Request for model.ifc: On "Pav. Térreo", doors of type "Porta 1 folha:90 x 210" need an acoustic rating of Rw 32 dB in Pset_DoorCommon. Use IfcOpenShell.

First a look at what the model holds.

```python
import ifcopenshell
import ifcopenshell.util.element

model = ifcopenshell.open("model.ifc")
print(model.schema)
storey = next(s for s in model.by_type("IfcBuildingStorey") if s.Name == "Pav. Térreo")
doors = [e for e in ifcopenshell.util.element.get_decomposition(storey) if e.is_a("IfcDoor")]
seen = {}
for e in doors:
    element_type = ifcopenshell.util.element.get_type(e)
    key = (element_type.Name if element_type != e and element_type else None, ifcopenshell.util.element.get_pset(e, "Pset_DoorCommon", "AcousticRating"))
    seen[key] = seen.get(key, 0) + 1
for (name, value), count in sorted(seen.items(), key=str):
    print(count, "x", name, "|", value)
```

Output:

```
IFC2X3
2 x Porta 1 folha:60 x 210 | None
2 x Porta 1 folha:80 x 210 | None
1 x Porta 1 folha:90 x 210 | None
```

```python
import ifcopenshell
import ifcopenshell.api.pset
import ifcopenshell.util.element

model = ifcopenshell.open("model.ifc")

storey = next(s for s in model.by_type("IfcBuildingStorey") if s.Name == "Pav. Térreo")
doors = [e for e in ifcopenshell.util.element.get_decomposition(storey) if e.is_a("IfcDoor")]

count = 0
for e in doors:
    element_type = ifcopenshell.util.element.get_type(e)
    if element_type in (None, e) or element_type.Name != "Porta 1 folha:90 x 210":
        continue
    # add_pset returns the element's existing set when there is one.
    pset = ifcopenshell.api.pset.add_pset(model, product=e, name="Pset_DoorCommon")
    ifcopenshell.api.pset.edit_pset(model, pset=pset, properties={"AcousticRating": "Rw 32 dB"})
    count += 1

print(count, "doors updated")

model.write("model_v2.ifc")
```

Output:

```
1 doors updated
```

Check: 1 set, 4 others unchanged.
